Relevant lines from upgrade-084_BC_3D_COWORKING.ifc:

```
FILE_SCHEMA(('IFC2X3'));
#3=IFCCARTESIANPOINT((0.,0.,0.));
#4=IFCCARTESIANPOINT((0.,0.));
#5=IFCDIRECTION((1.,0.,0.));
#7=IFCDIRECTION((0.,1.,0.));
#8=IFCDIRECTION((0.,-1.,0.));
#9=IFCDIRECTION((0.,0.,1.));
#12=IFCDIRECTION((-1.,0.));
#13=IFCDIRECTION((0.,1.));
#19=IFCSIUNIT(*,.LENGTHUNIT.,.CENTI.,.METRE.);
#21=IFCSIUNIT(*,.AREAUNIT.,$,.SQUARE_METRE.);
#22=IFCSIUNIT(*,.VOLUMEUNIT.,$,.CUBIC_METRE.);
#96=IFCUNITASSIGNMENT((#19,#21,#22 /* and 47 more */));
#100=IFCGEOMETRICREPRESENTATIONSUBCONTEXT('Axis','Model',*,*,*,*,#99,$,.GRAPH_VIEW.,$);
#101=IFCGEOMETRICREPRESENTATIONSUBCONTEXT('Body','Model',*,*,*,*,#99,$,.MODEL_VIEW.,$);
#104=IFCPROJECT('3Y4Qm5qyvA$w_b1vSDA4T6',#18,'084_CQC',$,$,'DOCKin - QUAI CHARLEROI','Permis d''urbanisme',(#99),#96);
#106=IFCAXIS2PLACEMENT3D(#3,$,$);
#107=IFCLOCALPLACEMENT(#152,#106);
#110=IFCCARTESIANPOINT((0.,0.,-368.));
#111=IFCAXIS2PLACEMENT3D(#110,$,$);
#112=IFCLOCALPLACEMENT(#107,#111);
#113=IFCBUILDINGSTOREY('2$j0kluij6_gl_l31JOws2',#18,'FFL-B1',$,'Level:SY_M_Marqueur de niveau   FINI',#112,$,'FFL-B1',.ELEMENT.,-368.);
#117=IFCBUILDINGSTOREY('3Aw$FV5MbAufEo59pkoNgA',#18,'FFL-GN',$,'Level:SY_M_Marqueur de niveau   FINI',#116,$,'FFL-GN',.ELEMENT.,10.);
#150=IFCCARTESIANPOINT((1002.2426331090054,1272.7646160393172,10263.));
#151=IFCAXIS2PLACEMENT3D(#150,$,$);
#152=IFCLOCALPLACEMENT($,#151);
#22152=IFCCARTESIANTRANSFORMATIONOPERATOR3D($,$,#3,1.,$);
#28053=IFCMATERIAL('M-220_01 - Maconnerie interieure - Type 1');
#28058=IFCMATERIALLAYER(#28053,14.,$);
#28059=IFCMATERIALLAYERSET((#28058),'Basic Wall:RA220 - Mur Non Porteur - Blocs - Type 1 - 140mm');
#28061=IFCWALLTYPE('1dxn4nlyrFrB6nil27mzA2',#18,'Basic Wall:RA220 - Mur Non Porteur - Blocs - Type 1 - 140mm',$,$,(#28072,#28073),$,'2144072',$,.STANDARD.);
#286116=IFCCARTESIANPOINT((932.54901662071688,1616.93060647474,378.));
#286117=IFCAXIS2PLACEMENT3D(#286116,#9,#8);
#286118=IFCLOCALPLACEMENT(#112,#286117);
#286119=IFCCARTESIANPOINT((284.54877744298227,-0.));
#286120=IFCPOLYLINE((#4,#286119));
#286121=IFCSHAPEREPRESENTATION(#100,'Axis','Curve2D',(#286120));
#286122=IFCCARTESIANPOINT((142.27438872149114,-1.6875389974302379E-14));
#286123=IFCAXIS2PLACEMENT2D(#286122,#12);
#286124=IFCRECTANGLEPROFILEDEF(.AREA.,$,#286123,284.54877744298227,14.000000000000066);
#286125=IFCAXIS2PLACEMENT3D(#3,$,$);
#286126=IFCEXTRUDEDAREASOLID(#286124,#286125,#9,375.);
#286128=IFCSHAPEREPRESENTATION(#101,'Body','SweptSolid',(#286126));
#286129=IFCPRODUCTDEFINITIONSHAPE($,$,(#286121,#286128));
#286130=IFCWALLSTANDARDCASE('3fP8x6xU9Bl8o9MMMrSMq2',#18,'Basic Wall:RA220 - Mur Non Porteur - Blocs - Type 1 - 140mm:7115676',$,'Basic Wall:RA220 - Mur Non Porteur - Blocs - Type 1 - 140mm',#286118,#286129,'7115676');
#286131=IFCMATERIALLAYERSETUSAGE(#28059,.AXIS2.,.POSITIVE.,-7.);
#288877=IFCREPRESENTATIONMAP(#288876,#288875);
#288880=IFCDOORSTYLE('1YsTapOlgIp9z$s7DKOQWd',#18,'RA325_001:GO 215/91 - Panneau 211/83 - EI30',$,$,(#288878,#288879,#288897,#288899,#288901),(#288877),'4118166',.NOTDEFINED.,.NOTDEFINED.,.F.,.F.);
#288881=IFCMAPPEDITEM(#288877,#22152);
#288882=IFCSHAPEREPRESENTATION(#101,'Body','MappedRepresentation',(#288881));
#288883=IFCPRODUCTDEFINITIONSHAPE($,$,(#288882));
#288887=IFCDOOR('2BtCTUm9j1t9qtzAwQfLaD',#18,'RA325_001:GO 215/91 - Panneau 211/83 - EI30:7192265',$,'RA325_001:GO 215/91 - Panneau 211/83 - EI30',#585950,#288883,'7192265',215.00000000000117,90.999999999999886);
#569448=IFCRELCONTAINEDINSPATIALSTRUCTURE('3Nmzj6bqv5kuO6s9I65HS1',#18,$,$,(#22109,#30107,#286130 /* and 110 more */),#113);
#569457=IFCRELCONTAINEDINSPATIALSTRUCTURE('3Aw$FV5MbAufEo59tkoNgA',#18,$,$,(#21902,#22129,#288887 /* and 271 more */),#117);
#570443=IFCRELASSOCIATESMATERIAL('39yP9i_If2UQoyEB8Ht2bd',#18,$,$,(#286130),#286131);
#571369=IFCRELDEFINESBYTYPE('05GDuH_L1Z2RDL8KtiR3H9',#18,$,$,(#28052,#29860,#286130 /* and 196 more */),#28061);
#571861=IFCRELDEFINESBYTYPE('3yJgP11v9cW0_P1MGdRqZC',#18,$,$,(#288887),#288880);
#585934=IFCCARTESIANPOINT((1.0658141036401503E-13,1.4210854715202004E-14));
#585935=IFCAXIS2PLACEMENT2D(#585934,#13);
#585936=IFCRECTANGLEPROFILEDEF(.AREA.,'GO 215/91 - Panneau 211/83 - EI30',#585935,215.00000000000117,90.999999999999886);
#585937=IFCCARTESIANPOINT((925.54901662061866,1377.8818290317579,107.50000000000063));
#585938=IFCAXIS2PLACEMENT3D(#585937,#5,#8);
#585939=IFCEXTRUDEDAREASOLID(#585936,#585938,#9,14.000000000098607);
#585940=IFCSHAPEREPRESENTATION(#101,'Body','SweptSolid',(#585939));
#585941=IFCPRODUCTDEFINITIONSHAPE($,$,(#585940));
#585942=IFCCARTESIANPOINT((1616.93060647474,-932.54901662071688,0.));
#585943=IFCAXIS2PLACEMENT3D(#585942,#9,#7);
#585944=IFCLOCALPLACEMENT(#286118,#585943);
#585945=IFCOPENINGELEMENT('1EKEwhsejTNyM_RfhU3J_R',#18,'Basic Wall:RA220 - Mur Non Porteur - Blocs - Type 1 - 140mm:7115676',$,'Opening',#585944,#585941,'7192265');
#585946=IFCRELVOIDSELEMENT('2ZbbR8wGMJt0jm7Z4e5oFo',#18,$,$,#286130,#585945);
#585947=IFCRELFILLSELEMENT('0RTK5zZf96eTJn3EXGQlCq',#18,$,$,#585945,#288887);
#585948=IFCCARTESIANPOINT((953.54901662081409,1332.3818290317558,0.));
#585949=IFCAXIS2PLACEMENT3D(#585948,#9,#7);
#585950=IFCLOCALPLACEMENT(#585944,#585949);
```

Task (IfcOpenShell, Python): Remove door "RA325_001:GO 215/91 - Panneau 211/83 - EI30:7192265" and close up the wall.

```python
import ifcopenshell
import ifcopenshell.api.feature
import ifcopenshell.api.root
import ifcopenshell.geom
import ifcopenshell.util.shape

model = ifcopenshell.open("upgrade-084_BC_3D_COWORKING.ifc")
settings = ifcopenshell.geom.settings()


def volume(element):
    """Net volume in cubic metres, openings subtracted."""
    shape = ifcopenshell.geom.create_shape(settings, element)
    return ifcopenshell.util.shape.get_volume(shape.geometry)


door = model.by_id(288887)
opening = door.FillsVoids[0].RelatingOpeningElement
wall = opening.VoidsElements[0].RelatingBuildingElement
before = volume(wall)

ifcopenshell.api.root.remove_product(model, product=door)
ifcopenshell.api.feature.remove_feature(model, feature=opening)

after = volume(wall)

print(f"wall volume {before:.3f} -> {after:.3f} m3")

model.write("upgrade-084_BC_3D_COWORKING_edited.ifc")
```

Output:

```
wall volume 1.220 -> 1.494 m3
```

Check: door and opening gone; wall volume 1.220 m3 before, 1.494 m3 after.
